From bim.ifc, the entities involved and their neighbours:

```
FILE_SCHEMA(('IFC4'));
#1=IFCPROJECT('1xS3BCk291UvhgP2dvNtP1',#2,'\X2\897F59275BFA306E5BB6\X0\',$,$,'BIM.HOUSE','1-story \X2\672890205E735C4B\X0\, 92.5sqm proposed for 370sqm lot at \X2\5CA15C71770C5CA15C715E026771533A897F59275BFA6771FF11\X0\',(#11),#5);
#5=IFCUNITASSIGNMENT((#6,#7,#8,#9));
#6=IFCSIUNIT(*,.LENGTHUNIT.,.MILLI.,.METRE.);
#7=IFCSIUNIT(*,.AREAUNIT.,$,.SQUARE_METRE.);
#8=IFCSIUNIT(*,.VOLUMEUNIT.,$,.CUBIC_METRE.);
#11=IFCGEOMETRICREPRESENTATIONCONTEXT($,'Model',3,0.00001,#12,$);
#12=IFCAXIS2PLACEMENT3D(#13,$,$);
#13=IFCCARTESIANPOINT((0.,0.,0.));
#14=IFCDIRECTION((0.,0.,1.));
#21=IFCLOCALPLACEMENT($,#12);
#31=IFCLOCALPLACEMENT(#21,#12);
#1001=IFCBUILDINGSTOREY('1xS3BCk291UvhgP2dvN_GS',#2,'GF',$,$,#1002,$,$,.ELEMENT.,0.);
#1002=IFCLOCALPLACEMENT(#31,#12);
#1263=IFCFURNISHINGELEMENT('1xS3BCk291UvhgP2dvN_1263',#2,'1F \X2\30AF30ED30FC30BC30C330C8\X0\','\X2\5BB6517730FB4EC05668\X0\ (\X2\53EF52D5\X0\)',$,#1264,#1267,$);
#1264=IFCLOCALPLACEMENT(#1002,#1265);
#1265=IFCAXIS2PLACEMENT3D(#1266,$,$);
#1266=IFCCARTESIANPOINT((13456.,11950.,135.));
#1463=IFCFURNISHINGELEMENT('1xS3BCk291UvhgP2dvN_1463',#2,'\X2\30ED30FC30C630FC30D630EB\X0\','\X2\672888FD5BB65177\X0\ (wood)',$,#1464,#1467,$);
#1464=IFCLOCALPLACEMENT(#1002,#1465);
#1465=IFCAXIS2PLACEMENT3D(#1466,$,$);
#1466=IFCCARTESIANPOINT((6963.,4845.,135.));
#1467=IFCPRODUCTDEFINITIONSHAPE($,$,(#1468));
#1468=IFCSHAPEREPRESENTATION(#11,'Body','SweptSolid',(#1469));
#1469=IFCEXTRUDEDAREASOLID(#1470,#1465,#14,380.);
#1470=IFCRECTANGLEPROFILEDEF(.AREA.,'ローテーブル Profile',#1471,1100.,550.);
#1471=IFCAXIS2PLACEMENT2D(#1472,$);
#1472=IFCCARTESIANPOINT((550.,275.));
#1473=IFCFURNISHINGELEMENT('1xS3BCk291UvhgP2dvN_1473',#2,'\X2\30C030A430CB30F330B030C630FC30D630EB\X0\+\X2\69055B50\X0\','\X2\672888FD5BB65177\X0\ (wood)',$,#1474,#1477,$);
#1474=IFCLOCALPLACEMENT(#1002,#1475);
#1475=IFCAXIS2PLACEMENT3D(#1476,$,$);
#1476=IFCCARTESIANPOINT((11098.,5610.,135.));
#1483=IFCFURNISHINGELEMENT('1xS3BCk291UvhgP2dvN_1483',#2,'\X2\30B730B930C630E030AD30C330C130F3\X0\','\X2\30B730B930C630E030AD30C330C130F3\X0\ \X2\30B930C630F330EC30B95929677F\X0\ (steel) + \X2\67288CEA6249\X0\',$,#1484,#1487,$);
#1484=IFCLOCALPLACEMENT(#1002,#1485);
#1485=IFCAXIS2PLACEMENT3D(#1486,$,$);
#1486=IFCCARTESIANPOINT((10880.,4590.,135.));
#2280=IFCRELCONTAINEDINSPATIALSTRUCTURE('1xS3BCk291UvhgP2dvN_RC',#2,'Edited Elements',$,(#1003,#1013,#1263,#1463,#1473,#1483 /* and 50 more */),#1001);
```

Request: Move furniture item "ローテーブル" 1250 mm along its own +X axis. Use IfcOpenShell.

```python
import ifcopenshell
import ifcopenshell.api.geometry
import ifcopenshell.util.placement
import ifcopenshell.util.unit

model = ifcopenshell.open("bim.ifc")
unit_scale = ifcopenshell.util.unit.calculate_unit_scale(model)

item = model.by_guid("1xS3BCk291UvhgP2dvN_1463")
matrix = ifcopenshell.util.placement.get_local_placement(item.ObjectPlacement)
matrix[:3, 3] += matrix[:3, 0] * 1.25 / unit_scale
ifcopenshell.api.geometry.edit_object_placement(model, product=item, matrix=matrix, is_si=False)

print(ifcopenshell.util.placement.get_local_placement(item.ObjectPlacement).round(3) + 0.0)

model.write("bim_v2.ifc")
```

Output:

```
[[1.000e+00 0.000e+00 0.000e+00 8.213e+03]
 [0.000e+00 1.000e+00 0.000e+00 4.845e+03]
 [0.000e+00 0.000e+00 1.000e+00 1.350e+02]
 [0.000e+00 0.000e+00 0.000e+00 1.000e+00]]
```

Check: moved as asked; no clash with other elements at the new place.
